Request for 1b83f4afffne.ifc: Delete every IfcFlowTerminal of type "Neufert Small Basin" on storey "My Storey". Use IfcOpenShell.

First a look at what the model holds.

```python
import ifcopenshell
import ifcopenshell.util.element

model = ifcopenshell.open("1b83f4afffne.ifc")
print(model.schema)
storey = next(s for s in model.by_type("IfcBuildingStorey") if s.Name == "My Storey")
terminals = [e for e in ifcopenshell.util.element.get_decomposition(storey) if e.is_a("IfcFlowTerminal")]
seen = {}
for e in terminals:
    element_type = ifcopenshell.util.element.get_type(e)
    name = element_type.Name if element_type not in (None, e) else None
    seen[name] = seen.get(name, 0) + 1
for name, count in sorted(seen.items(), key=str):
    print(count, "x", name)
```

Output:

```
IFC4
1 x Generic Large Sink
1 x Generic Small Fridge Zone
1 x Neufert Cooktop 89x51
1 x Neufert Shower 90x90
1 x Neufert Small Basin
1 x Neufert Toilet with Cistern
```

```python
import ifcopenshell
import ifcopenshell.api.root
import ifcopenshell.util.element

model = ifcopenshell.open("1b83f4afffne.ifc")

storey = next(s for s in model.by_type("IfcBuildingStorey") if s.Name == "My Storey")
terminals = [e for e in ifcopenshell.util.element.get_decomposition(storey) if e.is_a("IfcFlowTerminal")]
targets = [e for e in terminals if (t := ifcopenshell.util.element.get_type(e)) not in (None, e) and t.Name == "Neufert Small Basin"]

for e in targets:
    ifcopenshell.api.root.remove_product(model, product=e)
print(len(targets), "removed")

model.write("1b83f4afffne_edited.ifc")
```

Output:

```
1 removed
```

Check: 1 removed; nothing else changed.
